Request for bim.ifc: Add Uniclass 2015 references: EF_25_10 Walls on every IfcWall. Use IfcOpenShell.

First a look at what the model holds.

```python
import ifcopenshell

model = ifcopenshell.open("bim.ifc")
print(model.schema)
print("classifications:", [c.Name for c in model.by_type("IfcClassification")])
for ifc_class in ("IfcDoor", "IfcRoof", "IfcStair", "IfcWall", "IfcWindow"):
    print(ifc_class, len(model.by_type(ifc_class)))
```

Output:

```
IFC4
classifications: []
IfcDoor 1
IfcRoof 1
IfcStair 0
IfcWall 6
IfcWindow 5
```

```python
import ifcopenshell
import ifcopenshell.api.classification

model = ifcopenshell.open("bim.ifc")

system = ifcopenshell.api.classification.add_classification(model, classification="Uniclass 2015")

codes = {
    "IfcWall": ("EF_25_10", "Walls"),
}
for ifc_class, (code, name) in codes.items():
    products = model.by_type(ifc_class)
    ifcopenshell.api.classification.add_reference(
        model, products=products, classification=system, identification=code, name=name
    )
    print(code, len(products))

model.write("bim_updated.ifc")
```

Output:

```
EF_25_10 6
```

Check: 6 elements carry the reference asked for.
